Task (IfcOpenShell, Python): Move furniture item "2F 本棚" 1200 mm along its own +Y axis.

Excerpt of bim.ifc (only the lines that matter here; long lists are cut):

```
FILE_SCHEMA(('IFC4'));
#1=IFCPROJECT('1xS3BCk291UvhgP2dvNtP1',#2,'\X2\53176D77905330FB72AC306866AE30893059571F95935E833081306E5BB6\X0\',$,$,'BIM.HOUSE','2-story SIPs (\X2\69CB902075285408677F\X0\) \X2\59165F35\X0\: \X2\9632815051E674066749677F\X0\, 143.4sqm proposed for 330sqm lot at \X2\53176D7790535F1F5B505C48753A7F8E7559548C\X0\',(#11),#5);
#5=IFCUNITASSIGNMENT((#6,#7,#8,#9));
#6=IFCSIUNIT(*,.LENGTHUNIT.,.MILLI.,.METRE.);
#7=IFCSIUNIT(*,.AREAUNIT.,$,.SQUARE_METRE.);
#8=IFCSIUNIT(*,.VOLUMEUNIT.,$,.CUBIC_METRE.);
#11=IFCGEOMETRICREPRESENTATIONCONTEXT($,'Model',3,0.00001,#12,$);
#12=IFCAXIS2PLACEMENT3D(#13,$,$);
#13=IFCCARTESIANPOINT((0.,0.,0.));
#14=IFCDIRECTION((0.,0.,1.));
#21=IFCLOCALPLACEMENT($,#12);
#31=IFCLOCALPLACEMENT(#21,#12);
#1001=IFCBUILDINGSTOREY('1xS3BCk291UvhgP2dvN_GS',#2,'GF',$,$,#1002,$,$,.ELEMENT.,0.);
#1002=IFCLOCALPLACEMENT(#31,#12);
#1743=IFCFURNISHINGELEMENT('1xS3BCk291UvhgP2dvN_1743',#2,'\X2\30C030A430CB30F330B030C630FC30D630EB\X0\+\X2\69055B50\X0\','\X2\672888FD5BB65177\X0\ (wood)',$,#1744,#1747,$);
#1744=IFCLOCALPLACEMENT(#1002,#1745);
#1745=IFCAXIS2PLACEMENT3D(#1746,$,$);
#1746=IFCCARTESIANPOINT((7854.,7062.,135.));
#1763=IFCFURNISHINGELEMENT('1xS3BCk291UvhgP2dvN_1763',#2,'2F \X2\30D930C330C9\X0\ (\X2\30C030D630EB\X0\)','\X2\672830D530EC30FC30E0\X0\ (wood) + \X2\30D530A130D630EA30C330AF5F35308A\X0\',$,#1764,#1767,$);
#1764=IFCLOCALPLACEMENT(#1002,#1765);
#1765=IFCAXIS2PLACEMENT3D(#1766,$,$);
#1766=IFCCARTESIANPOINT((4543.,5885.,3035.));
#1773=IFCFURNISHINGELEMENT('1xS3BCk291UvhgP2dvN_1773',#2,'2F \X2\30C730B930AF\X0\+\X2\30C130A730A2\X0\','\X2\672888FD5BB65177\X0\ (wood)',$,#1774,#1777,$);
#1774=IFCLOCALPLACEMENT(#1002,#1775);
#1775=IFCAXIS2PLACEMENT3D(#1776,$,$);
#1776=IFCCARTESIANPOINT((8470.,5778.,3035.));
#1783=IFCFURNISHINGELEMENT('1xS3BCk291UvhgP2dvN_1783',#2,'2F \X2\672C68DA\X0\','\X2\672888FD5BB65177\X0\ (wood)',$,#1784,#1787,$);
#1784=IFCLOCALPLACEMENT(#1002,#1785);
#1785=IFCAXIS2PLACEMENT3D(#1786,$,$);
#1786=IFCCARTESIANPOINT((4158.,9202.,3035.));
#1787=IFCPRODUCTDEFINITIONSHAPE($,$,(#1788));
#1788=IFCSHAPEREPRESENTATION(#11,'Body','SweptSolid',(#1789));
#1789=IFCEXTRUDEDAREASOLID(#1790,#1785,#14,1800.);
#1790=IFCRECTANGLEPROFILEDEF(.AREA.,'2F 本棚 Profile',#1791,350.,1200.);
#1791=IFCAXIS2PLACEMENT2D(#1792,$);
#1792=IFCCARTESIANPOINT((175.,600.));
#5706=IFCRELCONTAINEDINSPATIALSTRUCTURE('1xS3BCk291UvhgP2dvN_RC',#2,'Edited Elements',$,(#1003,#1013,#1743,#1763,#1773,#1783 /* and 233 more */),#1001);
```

```python
import ifcopenshell
import ifcopenshell.api.geometry
import ifcopenshell.util.placement
import ifcopenshell.util.unit

model = ifcopenshell.open("bim.ifc")
unit_scale = ifcopenshell.util.unit.calculate_unit_scale(model)

item = model.by_guid("1xS3BCk291UvhgP2dvN_1783")
matrix = ifcopenshell.util.placement.get_local_placement(item.ObjectPlacement)
matrix[:3, 3] += matrix[:3, 1] * 1.2 / unit_scale
ifcopenshell.api.geometry.edit_object_placement(model, product=item, matrix=matrix, is_si=False)

print(ifcopenshell.util.placement.get_local_placement(item.ObjectPlacement).round(3) + 0.0)

model.write("bim_updated.ifc")
```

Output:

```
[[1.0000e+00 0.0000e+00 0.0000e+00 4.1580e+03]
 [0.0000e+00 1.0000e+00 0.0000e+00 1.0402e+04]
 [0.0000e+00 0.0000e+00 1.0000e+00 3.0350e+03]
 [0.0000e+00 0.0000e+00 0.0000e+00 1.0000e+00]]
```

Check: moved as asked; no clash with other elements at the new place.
